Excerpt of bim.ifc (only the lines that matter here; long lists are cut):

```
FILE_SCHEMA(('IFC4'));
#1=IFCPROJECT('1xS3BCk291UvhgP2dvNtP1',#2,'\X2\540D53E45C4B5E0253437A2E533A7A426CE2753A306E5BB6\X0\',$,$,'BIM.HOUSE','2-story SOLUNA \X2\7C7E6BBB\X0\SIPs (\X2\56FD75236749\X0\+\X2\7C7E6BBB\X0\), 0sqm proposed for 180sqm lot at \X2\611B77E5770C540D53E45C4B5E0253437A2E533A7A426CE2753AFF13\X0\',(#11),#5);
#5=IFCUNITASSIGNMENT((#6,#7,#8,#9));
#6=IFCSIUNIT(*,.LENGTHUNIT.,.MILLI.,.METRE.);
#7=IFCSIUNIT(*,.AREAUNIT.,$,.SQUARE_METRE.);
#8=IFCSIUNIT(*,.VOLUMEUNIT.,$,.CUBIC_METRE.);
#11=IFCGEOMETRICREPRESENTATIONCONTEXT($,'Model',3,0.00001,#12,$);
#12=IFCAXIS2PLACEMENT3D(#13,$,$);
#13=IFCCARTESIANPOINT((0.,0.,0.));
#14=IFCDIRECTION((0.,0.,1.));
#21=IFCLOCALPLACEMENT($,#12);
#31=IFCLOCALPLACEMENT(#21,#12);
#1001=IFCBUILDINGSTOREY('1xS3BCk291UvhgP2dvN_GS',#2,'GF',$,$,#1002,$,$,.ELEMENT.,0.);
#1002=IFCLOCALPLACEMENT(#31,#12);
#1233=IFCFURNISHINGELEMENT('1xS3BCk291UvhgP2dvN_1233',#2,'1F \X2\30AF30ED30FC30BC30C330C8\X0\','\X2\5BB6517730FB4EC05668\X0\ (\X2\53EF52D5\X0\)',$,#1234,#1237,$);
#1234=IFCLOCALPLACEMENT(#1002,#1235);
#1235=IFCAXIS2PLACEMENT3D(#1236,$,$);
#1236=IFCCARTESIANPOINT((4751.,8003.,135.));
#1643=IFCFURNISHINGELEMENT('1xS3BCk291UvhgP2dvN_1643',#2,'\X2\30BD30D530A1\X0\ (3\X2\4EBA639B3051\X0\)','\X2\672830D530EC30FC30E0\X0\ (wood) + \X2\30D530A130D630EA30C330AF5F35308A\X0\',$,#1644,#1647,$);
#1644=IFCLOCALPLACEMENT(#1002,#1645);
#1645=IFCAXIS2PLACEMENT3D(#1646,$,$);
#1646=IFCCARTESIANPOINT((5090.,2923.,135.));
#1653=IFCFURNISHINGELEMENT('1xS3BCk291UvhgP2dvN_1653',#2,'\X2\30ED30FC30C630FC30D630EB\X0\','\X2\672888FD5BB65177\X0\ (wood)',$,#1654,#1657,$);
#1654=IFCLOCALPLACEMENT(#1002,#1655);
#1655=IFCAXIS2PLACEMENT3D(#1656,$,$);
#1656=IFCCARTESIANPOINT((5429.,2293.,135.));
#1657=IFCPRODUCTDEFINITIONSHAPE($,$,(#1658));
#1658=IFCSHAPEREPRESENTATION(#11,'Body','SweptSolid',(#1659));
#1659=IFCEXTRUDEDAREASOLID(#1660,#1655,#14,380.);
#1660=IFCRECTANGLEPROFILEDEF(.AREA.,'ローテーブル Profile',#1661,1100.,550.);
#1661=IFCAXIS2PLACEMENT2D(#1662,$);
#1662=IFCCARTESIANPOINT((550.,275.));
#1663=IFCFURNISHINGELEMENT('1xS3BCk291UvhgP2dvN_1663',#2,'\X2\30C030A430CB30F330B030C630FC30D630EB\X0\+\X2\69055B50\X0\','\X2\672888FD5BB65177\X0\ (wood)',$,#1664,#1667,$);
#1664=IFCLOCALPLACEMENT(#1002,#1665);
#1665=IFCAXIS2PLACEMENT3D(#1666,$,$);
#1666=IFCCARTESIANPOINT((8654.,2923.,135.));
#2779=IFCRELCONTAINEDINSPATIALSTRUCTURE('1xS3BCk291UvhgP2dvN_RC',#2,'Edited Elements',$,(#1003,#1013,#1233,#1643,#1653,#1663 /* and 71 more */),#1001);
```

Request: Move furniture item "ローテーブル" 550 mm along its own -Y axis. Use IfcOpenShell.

```python
import ifcopenshell
import ifcopenshell.api.geometry
import ifcopenshell.util.placement

model = ifcopenshell.open("bim.ifc")

item = model.by_guid("1xS3BCk291UvhgP2dvN_1653")
matrix = ifcopenshell.util.placement.get_local_placement(item.ObjectPlacement)
matrix[:3, 3] -= matrix[:3, 1] * 550.0
ifcopenshell.api.geometry.edit_object_placement(model, product=item, matrix=matrix, is_si=False)

print(ifcopenshell.util.placement.get_local_placement(item.ObjectPlacement).round(3) + 0.0)

model.write("bim-out.ifc")
```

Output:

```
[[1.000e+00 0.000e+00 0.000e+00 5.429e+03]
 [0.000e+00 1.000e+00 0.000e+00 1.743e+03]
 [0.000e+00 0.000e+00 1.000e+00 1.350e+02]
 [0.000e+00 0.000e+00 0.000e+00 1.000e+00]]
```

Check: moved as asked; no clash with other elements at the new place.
